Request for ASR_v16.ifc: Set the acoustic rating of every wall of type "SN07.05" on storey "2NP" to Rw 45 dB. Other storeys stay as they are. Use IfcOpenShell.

First a look at what the model holds.

```python
import ifcopenshell
import ifcopenshell.util.element

model = ifcopenshell.open("ASR_v16.ifc")
print(model.schema)
storey = next(s for s in model.by_type("IfcBuildingStorey") if s.Name == "2NP")
walls = [e for e in ifcopenshell.util.element.get_decomposition(storey) if e.is_a("IfcWall")]
seen = {}
for e in walls:
    element_type = ifcopenshell.util.element.get_type(e)
    key = (element_type.Name if element_type != e and element_type else None, ifcopenshell.util.element.get_pset(e, "Pset_WallCommon", "AcousticRating"))
    seen[key] = seen.get(key, 0) + 1
for (name, value), count in sorted(seen.items(), key=str):
    print(count, "x", name, "|", value)
```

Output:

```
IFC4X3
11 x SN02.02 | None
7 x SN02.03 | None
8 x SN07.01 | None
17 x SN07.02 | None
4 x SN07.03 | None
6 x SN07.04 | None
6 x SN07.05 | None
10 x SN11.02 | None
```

```python
import ifcopenshell
import ifcopenshell.api.pset
import ifcopenshell.util.element

model = ifcopenshell.open("ASR_v16.ifc")

storey = next(s for s in model.by_type("IfcBuildingStorey") if s.Name == "2NP")
walls = [e for e in ifcopenshell.util.element.get_decomposition(storey) if e.is_a("IfcWall")]

count = 0
for e in walls:
    element_type = ifcopenshell.util.element.get_type(e)
    if element_type in (None, e) or element_type.Name != "SN07.05":
        continue
    # add_pset returns the element's existing set when there is one.
    pset = ifcopenshell.api.pset.add_pset(model, product=e, name="Pset_WallCommon")
    ifcopenshell.api.pset.edit_pset(model, pset=pset, properties={"AcousticRating": "Rw 45 dB"})
    count += 1

print(count, "walls updated")

model.write("ASR_v16_updated.ifc")
```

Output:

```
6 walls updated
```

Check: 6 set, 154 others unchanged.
